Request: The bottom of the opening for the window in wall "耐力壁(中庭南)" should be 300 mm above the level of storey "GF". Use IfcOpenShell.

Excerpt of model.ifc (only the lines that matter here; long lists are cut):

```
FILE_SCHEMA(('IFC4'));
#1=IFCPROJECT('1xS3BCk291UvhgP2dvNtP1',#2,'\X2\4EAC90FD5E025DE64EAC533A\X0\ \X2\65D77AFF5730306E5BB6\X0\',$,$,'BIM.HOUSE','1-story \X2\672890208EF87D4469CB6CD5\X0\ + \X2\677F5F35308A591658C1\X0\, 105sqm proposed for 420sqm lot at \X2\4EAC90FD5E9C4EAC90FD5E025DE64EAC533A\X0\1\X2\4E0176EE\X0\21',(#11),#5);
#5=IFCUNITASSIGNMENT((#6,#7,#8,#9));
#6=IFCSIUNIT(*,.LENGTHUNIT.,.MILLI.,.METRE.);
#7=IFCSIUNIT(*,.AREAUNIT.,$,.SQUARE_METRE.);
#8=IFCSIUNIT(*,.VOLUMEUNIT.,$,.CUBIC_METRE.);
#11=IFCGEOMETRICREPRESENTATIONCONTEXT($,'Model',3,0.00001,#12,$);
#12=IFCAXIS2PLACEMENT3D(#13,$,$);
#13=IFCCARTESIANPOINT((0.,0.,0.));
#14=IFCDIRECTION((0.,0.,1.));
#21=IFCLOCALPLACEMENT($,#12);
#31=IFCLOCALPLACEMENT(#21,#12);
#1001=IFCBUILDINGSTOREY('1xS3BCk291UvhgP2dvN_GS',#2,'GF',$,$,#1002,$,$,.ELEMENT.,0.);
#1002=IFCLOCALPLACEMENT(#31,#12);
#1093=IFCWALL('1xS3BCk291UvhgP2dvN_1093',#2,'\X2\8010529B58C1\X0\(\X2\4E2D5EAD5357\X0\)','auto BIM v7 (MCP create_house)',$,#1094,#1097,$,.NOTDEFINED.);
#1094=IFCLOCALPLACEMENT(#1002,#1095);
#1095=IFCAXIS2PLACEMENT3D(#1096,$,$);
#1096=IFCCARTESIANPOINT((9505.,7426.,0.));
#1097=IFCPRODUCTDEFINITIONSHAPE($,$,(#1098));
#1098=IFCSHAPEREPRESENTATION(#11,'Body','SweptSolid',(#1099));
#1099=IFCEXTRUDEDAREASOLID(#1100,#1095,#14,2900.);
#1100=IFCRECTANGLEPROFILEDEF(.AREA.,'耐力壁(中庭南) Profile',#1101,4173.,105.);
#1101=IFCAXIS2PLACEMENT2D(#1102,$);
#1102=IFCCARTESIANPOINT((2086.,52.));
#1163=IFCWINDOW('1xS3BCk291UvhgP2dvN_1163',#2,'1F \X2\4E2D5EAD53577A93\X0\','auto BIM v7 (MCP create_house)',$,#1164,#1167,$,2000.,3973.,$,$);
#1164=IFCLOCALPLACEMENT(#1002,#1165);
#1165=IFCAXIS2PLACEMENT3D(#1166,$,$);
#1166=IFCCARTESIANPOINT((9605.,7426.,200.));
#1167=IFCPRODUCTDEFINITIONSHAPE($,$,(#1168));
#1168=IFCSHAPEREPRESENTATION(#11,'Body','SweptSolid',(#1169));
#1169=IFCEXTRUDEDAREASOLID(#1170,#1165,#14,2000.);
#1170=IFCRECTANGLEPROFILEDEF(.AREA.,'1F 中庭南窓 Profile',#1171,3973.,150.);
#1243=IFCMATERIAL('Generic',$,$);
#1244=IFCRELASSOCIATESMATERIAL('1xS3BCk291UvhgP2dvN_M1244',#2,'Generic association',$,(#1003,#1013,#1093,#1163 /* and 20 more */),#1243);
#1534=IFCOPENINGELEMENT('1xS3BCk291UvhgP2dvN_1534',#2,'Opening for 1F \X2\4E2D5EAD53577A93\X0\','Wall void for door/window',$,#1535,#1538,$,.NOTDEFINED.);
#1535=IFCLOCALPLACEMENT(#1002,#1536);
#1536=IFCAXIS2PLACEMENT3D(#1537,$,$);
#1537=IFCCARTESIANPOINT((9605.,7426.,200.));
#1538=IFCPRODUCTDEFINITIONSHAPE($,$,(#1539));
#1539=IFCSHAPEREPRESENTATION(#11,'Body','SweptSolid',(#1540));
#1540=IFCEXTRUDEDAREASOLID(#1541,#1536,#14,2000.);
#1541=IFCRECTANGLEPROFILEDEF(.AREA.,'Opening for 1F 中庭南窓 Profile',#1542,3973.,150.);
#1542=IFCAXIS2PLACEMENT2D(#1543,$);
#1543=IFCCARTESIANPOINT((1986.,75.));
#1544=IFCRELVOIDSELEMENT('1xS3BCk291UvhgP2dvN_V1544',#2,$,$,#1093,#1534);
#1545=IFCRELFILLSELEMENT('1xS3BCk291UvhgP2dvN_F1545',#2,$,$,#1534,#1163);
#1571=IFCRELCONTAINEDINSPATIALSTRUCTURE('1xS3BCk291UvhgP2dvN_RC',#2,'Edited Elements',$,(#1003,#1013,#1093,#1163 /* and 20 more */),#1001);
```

```python
import numpy as np
import ifcopenshell
import ifcopenshell.api.geometry
import ifcopenshell.geom
import ifcopenshell.util.element
import ifcopenshell.util.placement
import ifcopenshell.util.shape
import ifcopenshell.util.unit

model = ifcopenshell.open("model.ifc")
unit_scale = ifcopenshell.util.unit.calculate_unit_scale(model)

window = model.by_guid("1xS3BCk291UvhgP2dvN_1163")
opening = window.FillsVoids[0].RelatingOpeningElement
storey = ifcopenshell.util.element.get_container(window, ifc_class="IfcBuildingStorey")
level = ifcopenshell.util.placement.get_local_placement(storey.ObjectPlacement)[2, 3]

# The opening's origin need not be at the sill, so measure its lowest point.
shape = ifcopenshell.geom.create_shape(ifcopenshell.geom.settings(), opening)
bottom = ifcopenshell.util.shape.get_shape_bottom_elevation(shape, shape.geometry) / unit_scale
dz = level + 0.3 / unit_scale - bottom

shift = np.array([0.0, 0.0, dz])
# The window is not placed relative to its opening, so move both.
for product in (opening, window):
    matrix = ifcopenshell.util.placement.get_local_placement(product.ObjectPlacement)
    matrix[:3, 3] += shift
    ifcopenshell.api.geometry.edit_object_placement(model, product=product, matrix=matrix, is_si=False)

print(f"moved by {dz * unit_scale:+.3f} m")

model.write("model_rev.ifc")
```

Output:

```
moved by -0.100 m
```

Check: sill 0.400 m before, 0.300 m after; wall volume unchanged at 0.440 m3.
